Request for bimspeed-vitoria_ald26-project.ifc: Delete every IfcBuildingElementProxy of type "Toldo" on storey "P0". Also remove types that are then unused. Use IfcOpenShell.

First a look at what the model holds.

```python
import ifcopenshell
import ifcopenshell.util.element

model = ifcopenshell.open("bimspeed-vitoria_ald26-project.ifc")
print(model.schema)
storey = next(s for s in model.by_type("IfcBuildingStorey") if s.Name == "P0")
proxies = [e for e in ifcopenshell.util.element.get_decomposition(storey) if e.is_a("IfcBuildingElementProxy")]
seen = {}
for e in proxies:
    element_type = ifcopenshell.util.element.get_type(e)
    name = element_type.Name if element_type not in (None, e) else None
    seen[name] = seen.get(name, 0) + 1
for name, count in sorted(seen.items(), key=str):
    print(count, "x", name)
```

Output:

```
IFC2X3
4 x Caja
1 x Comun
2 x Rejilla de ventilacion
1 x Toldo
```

```python
import ifcopenshell
import ifcopenshell.api.root
import ifcopenshell.util.element

model = ifcopenshell.open("bimspeed-vitoria_ald26-project.ifc")

storey = next(s for s in model.by_type("IfcBuildingStorey") if s.Name == "P0")
proxies = [e for e in ifcopenshell.util.element.get_decomposition(storey) if e.is_a("IfcBuildingElementProxy")]
targets = [e for e in proxies if (t := ifcopenshell.util.element.get_type(e)) not in (None, e) and t.Name == "Toldo"]
types = {ifcopenshell.util.element.get_type(e) for e in targets} - {None, *targets}

for e in targets:
    ifcopenshell.api.root.remove_product(model, product=e)
print(len(targets), "removed")

unused = [t for t in types if not ifcopenshell.util.element.get_types(t)]
for t in unused:
    ifcopenshell.api.root.remove_product(model, product=t)
print(len(unused), "unused types removed")

model.write("bimspeed-vitoria_ald26-project_v2.ifc")
```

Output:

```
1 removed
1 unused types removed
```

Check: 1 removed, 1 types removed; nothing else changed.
